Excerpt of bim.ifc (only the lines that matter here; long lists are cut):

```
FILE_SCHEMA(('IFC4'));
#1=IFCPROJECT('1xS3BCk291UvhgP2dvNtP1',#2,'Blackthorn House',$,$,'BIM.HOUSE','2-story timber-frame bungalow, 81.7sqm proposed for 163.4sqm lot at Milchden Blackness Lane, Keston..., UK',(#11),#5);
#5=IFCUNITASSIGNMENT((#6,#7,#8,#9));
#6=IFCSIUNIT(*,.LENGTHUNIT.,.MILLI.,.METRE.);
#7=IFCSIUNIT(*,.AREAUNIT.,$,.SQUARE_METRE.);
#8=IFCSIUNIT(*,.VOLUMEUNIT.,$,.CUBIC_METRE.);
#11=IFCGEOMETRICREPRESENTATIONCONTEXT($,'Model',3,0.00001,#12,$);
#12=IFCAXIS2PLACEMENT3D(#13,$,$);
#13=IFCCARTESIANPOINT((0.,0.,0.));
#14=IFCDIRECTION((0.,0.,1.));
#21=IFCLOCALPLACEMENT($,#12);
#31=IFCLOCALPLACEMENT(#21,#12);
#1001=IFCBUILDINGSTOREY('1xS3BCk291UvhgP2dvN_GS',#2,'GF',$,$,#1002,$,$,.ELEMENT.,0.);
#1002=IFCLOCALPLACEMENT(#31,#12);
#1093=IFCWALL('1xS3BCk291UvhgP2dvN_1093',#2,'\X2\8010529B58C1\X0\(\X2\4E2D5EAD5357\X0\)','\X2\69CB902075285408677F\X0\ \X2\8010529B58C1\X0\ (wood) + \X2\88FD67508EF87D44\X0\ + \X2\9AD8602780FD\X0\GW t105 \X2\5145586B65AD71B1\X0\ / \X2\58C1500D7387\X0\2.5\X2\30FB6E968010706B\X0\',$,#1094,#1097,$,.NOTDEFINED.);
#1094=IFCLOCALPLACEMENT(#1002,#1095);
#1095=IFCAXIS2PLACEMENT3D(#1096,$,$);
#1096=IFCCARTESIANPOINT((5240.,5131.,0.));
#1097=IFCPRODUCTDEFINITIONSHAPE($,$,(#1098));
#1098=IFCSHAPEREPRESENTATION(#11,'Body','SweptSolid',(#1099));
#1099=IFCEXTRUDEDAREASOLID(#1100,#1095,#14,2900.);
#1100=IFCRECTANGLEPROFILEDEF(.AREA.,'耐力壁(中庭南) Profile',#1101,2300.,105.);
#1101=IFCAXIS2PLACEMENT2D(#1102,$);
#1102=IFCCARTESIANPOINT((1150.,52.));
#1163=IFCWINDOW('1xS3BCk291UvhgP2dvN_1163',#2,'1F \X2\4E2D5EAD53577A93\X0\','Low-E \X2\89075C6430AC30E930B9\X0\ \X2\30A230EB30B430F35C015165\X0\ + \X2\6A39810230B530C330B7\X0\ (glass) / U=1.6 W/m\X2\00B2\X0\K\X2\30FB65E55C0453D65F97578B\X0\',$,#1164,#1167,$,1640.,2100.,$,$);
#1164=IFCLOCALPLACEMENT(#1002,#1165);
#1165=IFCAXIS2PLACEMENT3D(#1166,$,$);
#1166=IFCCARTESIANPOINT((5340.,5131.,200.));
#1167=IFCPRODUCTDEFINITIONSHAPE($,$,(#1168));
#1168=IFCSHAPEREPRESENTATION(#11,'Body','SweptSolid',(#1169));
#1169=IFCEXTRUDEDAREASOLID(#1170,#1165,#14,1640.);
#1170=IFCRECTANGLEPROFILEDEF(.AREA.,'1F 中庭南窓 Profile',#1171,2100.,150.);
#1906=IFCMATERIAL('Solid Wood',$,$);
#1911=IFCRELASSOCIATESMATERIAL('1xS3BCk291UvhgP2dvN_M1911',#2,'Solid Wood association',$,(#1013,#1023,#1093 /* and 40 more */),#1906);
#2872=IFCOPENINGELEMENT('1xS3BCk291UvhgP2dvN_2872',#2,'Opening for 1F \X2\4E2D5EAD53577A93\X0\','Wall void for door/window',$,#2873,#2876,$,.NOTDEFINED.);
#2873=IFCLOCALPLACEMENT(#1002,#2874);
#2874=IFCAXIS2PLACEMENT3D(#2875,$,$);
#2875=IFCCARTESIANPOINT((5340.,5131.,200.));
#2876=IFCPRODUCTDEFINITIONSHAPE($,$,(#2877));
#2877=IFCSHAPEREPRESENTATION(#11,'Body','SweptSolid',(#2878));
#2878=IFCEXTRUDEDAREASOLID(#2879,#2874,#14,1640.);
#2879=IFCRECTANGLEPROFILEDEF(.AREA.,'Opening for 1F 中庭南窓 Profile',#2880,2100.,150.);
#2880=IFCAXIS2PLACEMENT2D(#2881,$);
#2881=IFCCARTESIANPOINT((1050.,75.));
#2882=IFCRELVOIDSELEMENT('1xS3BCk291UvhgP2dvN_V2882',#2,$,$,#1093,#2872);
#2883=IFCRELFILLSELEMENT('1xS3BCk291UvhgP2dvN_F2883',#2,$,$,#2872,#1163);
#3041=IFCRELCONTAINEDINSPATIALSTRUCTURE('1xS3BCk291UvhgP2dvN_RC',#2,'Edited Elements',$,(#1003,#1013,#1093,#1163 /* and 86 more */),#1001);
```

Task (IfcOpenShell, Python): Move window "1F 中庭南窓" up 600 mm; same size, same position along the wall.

```python
import numpy as np
import ifcopenshell
import ifcopenshell.api.geometry
import ifcopenshell.util.placement
import ifcopenshell.util.unit

model = ifcopenshell.open("bim.ifc")
unit_scale = ifcopenshell.util.unit.calculate_unit_scale(model)

window = model.by_id(1163)
opening = window.FillsVoids[0].RelatingOpeningElement
dz = 0.6 / unit_scale

shift = np.array([0.0, 0.0, dz])
# The window is not placed relative to its opening, so move both.
for product in (opening, window):
    matrix = ifcopenshell.util.placement.get_local_placement(product.ObjectPlacement)
    matrix[:3, 3] += shift
    ifcopenshell.api.geometry.edit_object_placement(model, product=product, matrix=matrix, is_si=False)

print(f"moved by {dz * unit_scale:+.3f} m")

model.write("bim_updated.ifc")
```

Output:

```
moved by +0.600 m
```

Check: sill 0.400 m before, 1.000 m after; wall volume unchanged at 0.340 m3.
